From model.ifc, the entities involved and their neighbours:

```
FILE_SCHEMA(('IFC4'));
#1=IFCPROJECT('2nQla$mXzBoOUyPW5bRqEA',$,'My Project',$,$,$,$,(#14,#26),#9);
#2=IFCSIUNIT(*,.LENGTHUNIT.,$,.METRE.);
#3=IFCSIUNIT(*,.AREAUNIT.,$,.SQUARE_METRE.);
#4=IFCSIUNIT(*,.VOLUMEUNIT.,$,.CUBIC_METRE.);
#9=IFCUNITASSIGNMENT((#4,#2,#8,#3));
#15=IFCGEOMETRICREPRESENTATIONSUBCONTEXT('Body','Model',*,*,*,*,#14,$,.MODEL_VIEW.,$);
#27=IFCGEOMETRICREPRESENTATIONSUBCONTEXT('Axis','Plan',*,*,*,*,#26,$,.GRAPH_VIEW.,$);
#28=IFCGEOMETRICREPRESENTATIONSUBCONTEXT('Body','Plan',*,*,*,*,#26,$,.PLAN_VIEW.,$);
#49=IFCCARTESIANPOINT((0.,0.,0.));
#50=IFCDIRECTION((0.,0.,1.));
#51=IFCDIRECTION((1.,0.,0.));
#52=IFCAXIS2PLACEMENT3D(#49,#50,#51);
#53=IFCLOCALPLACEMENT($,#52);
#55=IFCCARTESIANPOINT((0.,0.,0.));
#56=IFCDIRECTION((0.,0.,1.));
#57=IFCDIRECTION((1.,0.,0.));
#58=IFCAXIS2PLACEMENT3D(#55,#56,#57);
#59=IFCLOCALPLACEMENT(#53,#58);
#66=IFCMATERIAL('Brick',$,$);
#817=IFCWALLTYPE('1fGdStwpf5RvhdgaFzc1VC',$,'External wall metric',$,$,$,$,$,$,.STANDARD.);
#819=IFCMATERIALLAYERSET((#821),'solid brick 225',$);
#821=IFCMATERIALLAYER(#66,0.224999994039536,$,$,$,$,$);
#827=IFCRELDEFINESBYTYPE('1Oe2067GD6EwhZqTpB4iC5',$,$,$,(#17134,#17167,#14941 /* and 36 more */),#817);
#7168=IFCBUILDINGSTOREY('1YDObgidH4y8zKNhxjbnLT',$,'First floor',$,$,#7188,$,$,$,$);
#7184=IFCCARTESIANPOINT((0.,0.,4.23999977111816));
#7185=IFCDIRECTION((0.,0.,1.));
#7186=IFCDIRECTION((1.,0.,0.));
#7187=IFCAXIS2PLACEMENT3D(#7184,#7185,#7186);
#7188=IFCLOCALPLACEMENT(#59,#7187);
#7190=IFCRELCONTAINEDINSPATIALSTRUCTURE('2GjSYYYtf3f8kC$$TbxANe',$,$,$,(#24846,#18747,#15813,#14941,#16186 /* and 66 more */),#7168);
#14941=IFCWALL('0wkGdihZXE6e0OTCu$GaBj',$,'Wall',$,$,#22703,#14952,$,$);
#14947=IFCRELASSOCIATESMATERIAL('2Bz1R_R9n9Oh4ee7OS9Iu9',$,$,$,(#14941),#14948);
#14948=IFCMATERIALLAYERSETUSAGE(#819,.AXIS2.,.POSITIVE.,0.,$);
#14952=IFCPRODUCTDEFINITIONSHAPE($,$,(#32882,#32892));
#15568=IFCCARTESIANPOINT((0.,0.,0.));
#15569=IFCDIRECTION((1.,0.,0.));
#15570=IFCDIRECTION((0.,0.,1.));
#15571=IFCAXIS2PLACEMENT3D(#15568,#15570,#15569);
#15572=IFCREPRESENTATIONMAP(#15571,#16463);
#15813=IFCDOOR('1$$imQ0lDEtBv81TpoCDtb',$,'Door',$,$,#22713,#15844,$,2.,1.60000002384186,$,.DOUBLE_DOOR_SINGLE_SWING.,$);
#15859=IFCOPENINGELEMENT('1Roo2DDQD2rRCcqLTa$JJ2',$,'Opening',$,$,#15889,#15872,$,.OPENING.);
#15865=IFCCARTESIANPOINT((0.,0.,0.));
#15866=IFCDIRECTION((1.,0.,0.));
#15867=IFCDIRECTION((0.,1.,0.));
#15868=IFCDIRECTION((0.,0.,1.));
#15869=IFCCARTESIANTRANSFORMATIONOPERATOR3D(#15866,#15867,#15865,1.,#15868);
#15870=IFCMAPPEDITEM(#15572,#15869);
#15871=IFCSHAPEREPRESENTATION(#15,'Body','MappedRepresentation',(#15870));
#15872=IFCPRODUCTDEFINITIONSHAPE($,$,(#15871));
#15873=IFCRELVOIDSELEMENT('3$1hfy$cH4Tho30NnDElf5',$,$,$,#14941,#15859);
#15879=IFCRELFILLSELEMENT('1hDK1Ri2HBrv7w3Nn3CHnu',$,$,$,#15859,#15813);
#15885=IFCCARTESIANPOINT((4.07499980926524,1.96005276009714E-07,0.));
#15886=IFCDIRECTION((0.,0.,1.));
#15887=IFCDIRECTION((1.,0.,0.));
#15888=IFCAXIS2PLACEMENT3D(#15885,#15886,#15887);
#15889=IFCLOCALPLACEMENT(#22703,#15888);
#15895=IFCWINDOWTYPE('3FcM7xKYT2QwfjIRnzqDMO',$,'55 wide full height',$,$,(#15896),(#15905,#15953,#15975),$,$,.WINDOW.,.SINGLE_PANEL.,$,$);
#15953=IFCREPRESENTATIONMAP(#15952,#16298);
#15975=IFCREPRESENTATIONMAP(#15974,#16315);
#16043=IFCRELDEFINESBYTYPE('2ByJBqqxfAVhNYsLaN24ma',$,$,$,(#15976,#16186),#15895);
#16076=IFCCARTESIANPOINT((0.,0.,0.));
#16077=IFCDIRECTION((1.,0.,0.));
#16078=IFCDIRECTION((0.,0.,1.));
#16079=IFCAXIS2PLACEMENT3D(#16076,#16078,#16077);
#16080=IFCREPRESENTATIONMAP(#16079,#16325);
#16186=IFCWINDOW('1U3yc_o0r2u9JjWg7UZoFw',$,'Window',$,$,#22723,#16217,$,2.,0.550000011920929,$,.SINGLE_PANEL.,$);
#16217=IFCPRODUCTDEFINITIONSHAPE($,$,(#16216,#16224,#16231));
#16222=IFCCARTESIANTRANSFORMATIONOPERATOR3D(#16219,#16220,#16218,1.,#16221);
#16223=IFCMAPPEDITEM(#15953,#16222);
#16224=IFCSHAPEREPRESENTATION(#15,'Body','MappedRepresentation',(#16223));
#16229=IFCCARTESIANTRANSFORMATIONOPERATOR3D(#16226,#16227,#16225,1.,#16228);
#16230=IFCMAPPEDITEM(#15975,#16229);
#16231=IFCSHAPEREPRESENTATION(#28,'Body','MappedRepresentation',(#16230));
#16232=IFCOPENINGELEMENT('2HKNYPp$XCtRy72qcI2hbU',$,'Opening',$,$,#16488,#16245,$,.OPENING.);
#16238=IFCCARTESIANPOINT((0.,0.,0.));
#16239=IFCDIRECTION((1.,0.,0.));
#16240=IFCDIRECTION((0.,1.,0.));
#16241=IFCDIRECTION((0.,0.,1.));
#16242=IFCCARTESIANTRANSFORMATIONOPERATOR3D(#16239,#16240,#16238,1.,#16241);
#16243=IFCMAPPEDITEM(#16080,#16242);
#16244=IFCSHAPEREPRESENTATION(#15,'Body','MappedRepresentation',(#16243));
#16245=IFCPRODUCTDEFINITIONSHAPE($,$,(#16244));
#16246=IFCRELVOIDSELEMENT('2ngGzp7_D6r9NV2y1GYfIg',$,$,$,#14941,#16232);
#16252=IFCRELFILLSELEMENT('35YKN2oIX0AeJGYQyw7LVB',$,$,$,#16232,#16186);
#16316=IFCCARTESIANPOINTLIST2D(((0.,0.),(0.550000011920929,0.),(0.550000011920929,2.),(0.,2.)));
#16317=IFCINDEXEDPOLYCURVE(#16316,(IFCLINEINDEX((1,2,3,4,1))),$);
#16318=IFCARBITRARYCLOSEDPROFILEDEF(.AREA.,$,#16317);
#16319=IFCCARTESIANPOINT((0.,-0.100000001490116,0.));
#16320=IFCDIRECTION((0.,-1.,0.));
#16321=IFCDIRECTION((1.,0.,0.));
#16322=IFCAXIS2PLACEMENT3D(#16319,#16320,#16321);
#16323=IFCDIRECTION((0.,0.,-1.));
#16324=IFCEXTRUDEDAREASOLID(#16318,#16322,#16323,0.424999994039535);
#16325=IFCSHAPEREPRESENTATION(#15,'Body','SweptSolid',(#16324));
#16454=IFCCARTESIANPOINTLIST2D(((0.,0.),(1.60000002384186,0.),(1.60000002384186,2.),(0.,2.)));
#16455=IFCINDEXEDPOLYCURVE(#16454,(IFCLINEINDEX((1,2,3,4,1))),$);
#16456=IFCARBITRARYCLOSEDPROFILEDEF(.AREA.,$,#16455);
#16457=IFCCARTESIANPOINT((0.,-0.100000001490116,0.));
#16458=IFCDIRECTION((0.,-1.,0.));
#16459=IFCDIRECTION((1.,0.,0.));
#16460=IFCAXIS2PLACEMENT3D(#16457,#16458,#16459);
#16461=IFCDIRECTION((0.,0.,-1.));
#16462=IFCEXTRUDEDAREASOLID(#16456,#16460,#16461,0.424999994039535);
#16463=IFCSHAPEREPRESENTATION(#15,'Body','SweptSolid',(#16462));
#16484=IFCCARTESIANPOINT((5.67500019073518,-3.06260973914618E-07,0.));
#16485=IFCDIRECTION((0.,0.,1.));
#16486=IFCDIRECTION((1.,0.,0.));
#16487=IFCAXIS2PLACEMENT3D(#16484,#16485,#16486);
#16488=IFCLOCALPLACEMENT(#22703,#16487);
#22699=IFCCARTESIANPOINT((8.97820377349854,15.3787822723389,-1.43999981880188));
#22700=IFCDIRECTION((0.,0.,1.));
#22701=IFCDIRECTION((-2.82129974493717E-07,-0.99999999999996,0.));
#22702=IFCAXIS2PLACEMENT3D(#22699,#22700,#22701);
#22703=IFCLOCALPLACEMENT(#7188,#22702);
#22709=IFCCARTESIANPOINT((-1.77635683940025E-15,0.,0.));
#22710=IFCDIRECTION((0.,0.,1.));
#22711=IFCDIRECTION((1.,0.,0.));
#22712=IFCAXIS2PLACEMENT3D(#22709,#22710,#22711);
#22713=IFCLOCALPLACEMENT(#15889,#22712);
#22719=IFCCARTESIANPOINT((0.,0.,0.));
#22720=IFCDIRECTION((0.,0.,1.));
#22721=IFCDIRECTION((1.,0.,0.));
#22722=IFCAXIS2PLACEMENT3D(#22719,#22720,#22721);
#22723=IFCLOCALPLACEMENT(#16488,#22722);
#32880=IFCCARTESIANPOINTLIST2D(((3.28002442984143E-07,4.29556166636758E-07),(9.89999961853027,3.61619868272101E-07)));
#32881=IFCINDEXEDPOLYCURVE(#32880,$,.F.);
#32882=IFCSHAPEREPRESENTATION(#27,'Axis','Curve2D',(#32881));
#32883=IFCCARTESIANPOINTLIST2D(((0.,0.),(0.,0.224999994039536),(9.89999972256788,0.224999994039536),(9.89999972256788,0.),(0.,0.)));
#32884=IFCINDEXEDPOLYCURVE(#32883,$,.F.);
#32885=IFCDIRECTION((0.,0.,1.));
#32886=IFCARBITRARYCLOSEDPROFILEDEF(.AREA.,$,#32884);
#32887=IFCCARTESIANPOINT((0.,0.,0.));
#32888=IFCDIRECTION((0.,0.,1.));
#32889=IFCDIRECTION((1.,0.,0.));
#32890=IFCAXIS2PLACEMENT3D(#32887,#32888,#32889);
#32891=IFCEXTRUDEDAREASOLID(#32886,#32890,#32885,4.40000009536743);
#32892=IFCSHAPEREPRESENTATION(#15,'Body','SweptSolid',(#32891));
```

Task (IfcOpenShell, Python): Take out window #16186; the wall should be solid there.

```python
import ifcopenshell
import ifcopenshell.api.feature
import ifcopenshell.api.root
import ifcopenshell.geom
import ifcopenshell.util.shape

model = ifcopenshell.open("model.ifc")
settings = ifcopenshell.geom.settings()


def volume(element):
    """Net volume in cubic metres, openings subtracted."""
    shape = ifcopenshell.geom.create_shape(settings, element)
    return ifcopenshell.util.shape.get_volume(shape.geometry)


window = model.by_guid("1U3yc_o0r2u9JjWg7UZoFw")
opening = window.FillsVoids[0].RelatingOpeningElement
wall = opening.VoidsElements[0].RelatingBuildingElement
before = volume(wall)

ifcopenshell.api.root.remove_product(model, product=window)
ifcopenshell.api.feature.remove_feature(model, feature=opening)

after = volume(wall)

print(f"wall volume {before:.3f} -> {after:.3f} m3")

model.write("model_rev.ifc")
```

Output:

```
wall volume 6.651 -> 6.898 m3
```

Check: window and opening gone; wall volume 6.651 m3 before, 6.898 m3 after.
